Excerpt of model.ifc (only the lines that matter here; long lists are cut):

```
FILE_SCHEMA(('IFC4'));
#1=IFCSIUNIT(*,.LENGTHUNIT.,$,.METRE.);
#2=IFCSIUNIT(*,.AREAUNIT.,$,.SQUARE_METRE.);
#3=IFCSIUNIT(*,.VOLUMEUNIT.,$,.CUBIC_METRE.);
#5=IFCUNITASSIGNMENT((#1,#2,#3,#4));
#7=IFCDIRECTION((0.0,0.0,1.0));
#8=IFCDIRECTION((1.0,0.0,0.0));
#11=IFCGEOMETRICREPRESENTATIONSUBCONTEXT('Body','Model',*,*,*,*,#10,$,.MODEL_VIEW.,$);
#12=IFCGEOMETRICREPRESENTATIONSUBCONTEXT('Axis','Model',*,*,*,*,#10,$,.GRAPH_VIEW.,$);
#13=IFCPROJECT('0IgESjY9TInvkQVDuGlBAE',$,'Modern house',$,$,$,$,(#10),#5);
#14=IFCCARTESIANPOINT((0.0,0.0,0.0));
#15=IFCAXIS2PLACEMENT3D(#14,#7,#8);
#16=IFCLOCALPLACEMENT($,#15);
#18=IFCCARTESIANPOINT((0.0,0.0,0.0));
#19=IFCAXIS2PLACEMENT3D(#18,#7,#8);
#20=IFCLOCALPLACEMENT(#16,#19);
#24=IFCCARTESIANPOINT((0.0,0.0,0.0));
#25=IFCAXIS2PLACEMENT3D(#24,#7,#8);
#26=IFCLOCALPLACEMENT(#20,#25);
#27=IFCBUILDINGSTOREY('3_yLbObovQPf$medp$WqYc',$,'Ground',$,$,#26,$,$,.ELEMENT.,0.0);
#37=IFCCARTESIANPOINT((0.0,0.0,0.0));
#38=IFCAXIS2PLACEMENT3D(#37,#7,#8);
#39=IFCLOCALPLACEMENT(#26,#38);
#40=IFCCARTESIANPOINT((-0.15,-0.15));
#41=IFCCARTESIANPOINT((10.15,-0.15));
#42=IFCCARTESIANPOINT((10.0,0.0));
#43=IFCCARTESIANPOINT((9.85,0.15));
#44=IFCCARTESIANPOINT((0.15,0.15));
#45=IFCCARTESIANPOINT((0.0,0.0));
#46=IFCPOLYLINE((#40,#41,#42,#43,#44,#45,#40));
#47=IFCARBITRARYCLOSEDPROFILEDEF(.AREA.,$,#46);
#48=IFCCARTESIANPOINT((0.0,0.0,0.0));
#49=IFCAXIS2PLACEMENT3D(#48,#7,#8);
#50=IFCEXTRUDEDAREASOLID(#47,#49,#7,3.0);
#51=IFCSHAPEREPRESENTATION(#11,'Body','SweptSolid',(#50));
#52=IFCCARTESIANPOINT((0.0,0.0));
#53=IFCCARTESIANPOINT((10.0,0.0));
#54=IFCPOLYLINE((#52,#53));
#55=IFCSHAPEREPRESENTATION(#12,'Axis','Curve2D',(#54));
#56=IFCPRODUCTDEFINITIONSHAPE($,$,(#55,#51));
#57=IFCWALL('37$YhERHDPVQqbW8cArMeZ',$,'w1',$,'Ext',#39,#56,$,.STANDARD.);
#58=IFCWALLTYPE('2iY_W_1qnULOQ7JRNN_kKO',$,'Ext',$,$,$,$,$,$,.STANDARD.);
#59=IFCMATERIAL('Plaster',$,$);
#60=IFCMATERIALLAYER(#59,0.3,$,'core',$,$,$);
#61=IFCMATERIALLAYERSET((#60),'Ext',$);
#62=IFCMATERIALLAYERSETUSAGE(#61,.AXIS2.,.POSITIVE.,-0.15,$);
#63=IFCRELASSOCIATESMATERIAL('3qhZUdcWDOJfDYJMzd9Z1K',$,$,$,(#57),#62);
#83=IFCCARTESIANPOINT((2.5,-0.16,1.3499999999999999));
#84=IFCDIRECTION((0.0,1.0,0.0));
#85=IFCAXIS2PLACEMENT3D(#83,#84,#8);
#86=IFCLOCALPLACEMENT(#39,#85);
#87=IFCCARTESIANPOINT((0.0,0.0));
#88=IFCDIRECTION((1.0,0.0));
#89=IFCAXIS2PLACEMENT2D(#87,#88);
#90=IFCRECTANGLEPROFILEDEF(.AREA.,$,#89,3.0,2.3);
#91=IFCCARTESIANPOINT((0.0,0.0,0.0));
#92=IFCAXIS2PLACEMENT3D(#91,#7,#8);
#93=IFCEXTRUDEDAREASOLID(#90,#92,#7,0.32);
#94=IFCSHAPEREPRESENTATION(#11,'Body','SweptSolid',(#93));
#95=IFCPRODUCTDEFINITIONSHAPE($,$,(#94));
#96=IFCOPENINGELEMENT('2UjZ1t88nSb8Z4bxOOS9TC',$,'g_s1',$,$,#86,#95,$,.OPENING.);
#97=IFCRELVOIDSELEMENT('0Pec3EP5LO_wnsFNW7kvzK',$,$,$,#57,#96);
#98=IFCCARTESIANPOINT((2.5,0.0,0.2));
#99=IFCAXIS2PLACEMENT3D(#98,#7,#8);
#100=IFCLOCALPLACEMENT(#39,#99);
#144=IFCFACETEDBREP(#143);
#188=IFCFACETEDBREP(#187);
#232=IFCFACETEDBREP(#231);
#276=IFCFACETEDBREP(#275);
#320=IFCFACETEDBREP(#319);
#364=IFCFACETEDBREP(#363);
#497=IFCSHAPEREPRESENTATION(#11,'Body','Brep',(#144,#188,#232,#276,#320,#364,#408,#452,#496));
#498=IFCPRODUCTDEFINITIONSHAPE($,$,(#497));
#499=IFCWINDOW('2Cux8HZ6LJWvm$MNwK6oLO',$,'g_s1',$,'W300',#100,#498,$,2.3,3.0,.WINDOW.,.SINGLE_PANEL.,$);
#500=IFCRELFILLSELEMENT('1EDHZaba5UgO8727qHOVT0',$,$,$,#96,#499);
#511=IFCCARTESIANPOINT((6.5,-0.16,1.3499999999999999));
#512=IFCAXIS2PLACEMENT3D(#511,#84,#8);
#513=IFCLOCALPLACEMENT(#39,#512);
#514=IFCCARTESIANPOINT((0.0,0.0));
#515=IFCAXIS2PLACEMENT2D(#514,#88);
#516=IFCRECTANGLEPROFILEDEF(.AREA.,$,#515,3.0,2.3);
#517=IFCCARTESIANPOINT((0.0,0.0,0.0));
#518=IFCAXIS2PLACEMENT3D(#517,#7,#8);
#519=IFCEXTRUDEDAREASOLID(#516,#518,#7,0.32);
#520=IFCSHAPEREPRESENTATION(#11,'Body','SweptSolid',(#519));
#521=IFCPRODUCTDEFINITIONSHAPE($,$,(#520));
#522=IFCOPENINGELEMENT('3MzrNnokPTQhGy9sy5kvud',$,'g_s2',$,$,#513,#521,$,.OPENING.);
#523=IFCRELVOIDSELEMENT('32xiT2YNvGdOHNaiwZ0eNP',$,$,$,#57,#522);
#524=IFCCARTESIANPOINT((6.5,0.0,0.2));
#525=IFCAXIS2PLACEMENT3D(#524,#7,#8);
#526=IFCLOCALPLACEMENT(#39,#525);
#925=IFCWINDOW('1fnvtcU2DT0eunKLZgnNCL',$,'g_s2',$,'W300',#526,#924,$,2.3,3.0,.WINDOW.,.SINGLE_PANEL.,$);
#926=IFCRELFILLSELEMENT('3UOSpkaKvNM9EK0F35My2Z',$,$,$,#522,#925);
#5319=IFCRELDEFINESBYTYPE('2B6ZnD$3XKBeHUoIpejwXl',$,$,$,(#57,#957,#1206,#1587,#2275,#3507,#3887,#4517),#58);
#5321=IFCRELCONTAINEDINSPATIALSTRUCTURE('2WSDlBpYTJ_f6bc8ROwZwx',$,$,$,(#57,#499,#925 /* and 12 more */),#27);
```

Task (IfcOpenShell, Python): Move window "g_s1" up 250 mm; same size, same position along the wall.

```python
import numpy as np
import ifcopenshell
import ifcopenshell.api.geometry
import ifcopenshell.util.placement
import ifcopenshell.util.unit

model = ifcopenshell.open("model.ifc")
unit_scale = ifcopenshell.util.unit.calculate_unit_scale(model)

window = model.by_guid("2Cux8HZ6LJWvm$MNwK6oLO")
opening = window.FillsVoids[0].RelatingOpeningElement
dz = 0.25

shift = np.array([0.0, 0.0, dz])
# The window is not placed relative to its opening, so move both.
for product in (opening, window):
    matrix = ifcopenshell.util.placement.get_local_placement(product.ObjectPlacement)
    matrix[:3, 3] += shift
    ifcopenshell.api.geometry.edit_object_placement(model, product=product, matrix=matrix, is_si=False)

print(f"moved by {dz * unit_scale:+.3f} m")

model.write("model-out.ifc")
```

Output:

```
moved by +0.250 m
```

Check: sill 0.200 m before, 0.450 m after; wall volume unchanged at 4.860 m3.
